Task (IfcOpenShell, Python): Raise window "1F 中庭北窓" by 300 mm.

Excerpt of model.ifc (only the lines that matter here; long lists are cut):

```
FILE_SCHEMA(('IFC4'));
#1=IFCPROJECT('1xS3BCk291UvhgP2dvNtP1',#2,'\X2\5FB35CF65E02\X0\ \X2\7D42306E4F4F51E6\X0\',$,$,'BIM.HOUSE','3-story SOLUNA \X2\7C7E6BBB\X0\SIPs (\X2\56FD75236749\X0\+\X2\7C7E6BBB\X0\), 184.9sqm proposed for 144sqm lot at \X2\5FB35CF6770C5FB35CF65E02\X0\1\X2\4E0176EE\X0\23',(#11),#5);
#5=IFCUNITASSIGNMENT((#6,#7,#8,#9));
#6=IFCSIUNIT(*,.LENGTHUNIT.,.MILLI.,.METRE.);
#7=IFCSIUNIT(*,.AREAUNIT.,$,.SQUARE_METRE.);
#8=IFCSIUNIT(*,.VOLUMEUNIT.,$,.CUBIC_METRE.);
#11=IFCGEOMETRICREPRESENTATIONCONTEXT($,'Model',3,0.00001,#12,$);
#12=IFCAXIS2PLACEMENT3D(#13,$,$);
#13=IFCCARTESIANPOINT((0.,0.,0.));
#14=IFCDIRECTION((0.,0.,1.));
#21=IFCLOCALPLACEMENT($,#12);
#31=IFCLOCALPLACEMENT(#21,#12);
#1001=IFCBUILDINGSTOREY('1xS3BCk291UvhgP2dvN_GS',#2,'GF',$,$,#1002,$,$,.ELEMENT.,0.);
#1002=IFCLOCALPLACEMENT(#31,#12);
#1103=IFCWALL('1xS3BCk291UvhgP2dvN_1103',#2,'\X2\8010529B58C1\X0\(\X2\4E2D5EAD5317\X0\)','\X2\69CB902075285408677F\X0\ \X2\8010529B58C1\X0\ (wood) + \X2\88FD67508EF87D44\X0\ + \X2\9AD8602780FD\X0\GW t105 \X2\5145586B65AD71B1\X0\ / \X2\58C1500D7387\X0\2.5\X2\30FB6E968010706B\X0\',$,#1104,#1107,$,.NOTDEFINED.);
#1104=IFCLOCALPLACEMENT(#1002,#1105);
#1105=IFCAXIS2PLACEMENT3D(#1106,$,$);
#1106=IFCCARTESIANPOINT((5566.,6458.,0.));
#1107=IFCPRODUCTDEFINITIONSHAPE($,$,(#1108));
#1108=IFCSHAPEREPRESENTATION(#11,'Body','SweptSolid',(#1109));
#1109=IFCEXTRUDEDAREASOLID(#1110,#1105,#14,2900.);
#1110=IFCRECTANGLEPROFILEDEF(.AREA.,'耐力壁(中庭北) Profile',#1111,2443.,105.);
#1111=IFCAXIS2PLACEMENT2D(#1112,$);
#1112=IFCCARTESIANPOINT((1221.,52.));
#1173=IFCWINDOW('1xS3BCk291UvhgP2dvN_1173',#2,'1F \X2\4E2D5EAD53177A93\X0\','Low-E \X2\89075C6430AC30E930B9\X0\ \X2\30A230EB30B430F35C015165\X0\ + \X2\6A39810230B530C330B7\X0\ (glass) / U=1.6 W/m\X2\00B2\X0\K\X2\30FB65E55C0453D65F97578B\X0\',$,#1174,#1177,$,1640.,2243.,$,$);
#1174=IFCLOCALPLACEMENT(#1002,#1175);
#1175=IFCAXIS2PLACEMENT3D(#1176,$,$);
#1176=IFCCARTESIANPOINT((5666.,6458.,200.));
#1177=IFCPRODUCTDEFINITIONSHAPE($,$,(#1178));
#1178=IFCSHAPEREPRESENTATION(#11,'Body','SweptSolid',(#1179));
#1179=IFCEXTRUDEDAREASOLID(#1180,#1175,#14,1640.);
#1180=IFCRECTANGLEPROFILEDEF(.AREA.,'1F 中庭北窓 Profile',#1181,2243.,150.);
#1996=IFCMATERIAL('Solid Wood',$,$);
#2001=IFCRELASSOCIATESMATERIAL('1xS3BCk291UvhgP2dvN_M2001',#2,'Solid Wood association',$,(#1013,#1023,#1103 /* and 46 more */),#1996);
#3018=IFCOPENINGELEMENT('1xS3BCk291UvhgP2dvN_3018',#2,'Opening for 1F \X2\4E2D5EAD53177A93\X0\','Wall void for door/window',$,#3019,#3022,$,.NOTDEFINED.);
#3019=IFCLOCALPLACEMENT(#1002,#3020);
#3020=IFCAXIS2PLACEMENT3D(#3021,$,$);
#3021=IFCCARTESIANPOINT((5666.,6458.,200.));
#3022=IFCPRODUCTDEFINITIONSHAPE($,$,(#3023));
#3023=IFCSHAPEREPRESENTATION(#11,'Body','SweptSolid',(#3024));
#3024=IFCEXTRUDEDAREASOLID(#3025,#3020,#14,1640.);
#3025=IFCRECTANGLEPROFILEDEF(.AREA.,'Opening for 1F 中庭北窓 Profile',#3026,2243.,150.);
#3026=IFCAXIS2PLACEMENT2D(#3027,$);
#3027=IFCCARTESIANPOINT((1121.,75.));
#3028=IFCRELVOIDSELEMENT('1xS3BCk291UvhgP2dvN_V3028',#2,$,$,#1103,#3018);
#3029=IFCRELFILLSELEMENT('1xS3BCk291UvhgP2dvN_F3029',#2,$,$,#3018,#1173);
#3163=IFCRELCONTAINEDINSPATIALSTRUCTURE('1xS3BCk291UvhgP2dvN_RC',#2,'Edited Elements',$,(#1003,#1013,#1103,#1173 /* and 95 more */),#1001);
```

```python
import numpy as np
import ifcopenshell
import ifcopenshell.api.geometry
import ifcopenshell.util.placement
import ifcopenshell.util.unit

model = ifcopenshell.open("model.ifc")
unit_scale = ifcopenshell.util.unit.calculate_unit_scale(model)

window = model.by_id(1173)
opening = window.FillsVoids[0].RelatingOpeningElement
dz = 0.3 / unit_scale

shift = np.array([0.0, 0.0, dz])
# The window is not placed relative to its opening, so move both.
for product in (opening, window):
    matrix = ifcopenshell.util.placement.get_local_placement(product.ObjectPlacement)
    matrix[:3, 3] += shift
    ifcopenshell.api.geometry.edit_object_placement(model, product=product, matrix=matrix, is_si=False)

print(f"moved by {dz * unit_scale:+.3f} m")

model.write("model_rev.ifc")
```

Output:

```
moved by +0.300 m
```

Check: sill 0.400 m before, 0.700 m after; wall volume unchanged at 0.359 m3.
